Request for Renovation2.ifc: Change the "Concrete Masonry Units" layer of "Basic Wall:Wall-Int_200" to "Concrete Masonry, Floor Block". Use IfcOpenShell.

First a look at what the model holds.

```python
import ifcopenshell
import ifcopenshell.util.element

model = ifcopenshell.open("Renovation2.ifc")
print(model.schema)
for layer_set in model.by_type("IfcMaterialLayerSet"):
    if layer_set.LayerSetName == "Basic Wall:Wall-Int_200":
        for layer in layer_set.MaterialLayers:
            print(layer.id(), layer.Material and layer.Material.Name, layer.LayerThickness, sep=" | ")
        print(len(ifcopenshell.util.element.get_elements_by_material(model, layer_set)), "elements and types use it")
print(sorted(m.Name for m in model.by_type("IfcMaterial") if m.Name)[:60])
```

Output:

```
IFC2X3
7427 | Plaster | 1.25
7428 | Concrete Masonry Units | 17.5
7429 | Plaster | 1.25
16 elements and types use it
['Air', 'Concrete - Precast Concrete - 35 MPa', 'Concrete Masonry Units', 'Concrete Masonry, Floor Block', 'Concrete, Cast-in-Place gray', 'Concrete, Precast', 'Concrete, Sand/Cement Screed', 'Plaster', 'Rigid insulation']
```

```python
import ifcopenshell
import ifcopenshell.api.material

model = ifcopenshell.open("Renovation2.ifc")

layer_set = next(s for s in model.by_type("IfcMaterialLayerSet") if s.LayerSetName == "Basic Wall:Wall-Int_200")
layer = next(l for l in layer_set.MaterialLayers if l.Material and l.Material.Name == "Concrete Masonry Units")
material = next(m for m in model.by_type("IfcMaterial") if m.Name == "Concrete Masonry, Floor Block")

# Point this one layer at the other material; renaming the old one would change it everywhere.
ifcopenshell.api.material.edit_layer(model, layer=layer, attributes={}, material=material)

print([l.Material.Name if l.Material else None for l in layer_set.MaterialLayers])

model.write("Renovation2_updated.ifc")
```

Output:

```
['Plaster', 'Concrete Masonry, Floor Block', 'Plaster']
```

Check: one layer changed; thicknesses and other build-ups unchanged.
